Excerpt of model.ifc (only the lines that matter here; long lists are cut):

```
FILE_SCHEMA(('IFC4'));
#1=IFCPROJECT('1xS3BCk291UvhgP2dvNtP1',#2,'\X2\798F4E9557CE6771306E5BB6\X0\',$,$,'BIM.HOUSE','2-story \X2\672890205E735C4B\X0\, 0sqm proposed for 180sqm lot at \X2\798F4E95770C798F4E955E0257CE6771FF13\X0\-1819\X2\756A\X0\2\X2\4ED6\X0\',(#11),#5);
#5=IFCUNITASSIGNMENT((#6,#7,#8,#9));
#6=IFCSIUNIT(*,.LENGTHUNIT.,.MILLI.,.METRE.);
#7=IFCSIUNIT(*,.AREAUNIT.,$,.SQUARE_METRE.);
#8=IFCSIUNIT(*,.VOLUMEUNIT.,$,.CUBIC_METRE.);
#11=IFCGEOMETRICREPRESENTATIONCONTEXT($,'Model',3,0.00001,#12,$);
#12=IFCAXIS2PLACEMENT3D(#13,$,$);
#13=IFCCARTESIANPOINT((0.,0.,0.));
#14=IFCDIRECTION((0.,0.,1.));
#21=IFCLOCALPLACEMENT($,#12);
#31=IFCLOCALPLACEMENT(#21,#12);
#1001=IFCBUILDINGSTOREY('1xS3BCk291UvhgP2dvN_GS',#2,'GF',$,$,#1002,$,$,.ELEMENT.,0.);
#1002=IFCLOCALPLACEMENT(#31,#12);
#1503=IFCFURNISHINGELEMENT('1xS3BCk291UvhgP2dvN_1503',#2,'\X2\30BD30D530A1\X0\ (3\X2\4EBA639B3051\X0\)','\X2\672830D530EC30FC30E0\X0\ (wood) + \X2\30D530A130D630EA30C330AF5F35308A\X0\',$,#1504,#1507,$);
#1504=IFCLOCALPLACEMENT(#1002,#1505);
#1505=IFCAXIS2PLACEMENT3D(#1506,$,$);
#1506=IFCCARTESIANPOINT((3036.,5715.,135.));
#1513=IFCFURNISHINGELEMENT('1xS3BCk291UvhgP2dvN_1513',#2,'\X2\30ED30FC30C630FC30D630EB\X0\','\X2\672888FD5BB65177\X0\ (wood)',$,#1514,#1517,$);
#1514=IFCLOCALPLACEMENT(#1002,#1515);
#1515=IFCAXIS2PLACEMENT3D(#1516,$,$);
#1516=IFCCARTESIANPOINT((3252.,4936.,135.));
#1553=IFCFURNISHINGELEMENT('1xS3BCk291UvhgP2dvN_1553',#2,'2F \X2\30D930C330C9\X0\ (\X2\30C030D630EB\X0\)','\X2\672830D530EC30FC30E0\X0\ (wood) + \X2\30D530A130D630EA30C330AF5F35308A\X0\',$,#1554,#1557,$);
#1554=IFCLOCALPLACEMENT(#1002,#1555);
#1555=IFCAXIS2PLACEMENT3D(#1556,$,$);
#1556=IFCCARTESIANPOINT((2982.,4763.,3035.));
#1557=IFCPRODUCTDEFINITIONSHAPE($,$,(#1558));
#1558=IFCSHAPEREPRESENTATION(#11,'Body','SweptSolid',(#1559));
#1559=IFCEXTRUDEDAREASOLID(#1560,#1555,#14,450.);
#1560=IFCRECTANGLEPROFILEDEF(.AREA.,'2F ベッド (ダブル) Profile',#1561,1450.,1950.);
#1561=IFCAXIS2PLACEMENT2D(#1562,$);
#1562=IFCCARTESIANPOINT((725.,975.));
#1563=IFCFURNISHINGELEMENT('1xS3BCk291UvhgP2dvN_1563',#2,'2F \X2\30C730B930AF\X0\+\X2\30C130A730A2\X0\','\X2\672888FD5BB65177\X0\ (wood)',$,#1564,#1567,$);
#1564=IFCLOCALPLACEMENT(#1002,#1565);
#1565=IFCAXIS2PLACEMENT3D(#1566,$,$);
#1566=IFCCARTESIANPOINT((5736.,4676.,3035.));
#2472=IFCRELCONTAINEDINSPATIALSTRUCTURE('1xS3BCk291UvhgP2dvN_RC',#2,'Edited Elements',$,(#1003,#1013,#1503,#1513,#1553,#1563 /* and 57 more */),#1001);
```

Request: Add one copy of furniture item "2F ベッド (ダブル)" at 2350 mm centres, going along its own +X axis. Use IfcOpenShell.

```python
import ifcopenshell
import ifcopenshell.api.geometry
import ifcopenshell.api.root
import ifcopenshell.util.element
import ifcopenshell.util.placement
import ifcopenshell.util.unit

model = ifcopenshell.open("model.ifc")
unit_scale = ifcopenshell.util.unit.calculate_unit_scale(model)


def reuse_history(source, copy):
    """copy_class also copies each property set's owner history, people and application; keep the originals."""
    for rel in copy.IsDefinedBy:
        if rel.is_a("IfcRelDefinesByProperties") and (history := rel.RelatingPropertyDefinition.OwnerHistory):
            rel.RelatingPropertyDefinition.OwnerHistory = source.OwnerHistory
            ifcopenshell.util.element.remove_deep2(model, history)


source = model.by_guid("1xS3BCk291UvhgP2dvN_1553")
base = ifcopenshell.util.placement.get_local_placement(source.ObjectPlacement)
step = base[:3, 0] * 2.35 / unit_scale

for i in range(1, 2):
    copy = ifcopenshell.api.root.copy_class(model, product=source)
    copy.Representation = ifcopenshell.util.element.copy_deep(
        model, source.Representation, exclude=["IfcGeometricRepresentationContext", "IfcRepresentationMap"]
    )
    reuse_history(source, copy)
    matrix = base.copy()
    matrix[:3, 3] += i * step
    print("added at", matrix[:3, 3].round(3) + 0.0)
    ifcopenshell.api.geometry.edit_object_placement(model, product=copy, matrix=matrix, is_si=False)

model.write("model_rev.ifc")
```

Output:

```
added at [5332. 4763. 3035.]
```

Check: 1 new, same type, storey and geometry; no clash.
